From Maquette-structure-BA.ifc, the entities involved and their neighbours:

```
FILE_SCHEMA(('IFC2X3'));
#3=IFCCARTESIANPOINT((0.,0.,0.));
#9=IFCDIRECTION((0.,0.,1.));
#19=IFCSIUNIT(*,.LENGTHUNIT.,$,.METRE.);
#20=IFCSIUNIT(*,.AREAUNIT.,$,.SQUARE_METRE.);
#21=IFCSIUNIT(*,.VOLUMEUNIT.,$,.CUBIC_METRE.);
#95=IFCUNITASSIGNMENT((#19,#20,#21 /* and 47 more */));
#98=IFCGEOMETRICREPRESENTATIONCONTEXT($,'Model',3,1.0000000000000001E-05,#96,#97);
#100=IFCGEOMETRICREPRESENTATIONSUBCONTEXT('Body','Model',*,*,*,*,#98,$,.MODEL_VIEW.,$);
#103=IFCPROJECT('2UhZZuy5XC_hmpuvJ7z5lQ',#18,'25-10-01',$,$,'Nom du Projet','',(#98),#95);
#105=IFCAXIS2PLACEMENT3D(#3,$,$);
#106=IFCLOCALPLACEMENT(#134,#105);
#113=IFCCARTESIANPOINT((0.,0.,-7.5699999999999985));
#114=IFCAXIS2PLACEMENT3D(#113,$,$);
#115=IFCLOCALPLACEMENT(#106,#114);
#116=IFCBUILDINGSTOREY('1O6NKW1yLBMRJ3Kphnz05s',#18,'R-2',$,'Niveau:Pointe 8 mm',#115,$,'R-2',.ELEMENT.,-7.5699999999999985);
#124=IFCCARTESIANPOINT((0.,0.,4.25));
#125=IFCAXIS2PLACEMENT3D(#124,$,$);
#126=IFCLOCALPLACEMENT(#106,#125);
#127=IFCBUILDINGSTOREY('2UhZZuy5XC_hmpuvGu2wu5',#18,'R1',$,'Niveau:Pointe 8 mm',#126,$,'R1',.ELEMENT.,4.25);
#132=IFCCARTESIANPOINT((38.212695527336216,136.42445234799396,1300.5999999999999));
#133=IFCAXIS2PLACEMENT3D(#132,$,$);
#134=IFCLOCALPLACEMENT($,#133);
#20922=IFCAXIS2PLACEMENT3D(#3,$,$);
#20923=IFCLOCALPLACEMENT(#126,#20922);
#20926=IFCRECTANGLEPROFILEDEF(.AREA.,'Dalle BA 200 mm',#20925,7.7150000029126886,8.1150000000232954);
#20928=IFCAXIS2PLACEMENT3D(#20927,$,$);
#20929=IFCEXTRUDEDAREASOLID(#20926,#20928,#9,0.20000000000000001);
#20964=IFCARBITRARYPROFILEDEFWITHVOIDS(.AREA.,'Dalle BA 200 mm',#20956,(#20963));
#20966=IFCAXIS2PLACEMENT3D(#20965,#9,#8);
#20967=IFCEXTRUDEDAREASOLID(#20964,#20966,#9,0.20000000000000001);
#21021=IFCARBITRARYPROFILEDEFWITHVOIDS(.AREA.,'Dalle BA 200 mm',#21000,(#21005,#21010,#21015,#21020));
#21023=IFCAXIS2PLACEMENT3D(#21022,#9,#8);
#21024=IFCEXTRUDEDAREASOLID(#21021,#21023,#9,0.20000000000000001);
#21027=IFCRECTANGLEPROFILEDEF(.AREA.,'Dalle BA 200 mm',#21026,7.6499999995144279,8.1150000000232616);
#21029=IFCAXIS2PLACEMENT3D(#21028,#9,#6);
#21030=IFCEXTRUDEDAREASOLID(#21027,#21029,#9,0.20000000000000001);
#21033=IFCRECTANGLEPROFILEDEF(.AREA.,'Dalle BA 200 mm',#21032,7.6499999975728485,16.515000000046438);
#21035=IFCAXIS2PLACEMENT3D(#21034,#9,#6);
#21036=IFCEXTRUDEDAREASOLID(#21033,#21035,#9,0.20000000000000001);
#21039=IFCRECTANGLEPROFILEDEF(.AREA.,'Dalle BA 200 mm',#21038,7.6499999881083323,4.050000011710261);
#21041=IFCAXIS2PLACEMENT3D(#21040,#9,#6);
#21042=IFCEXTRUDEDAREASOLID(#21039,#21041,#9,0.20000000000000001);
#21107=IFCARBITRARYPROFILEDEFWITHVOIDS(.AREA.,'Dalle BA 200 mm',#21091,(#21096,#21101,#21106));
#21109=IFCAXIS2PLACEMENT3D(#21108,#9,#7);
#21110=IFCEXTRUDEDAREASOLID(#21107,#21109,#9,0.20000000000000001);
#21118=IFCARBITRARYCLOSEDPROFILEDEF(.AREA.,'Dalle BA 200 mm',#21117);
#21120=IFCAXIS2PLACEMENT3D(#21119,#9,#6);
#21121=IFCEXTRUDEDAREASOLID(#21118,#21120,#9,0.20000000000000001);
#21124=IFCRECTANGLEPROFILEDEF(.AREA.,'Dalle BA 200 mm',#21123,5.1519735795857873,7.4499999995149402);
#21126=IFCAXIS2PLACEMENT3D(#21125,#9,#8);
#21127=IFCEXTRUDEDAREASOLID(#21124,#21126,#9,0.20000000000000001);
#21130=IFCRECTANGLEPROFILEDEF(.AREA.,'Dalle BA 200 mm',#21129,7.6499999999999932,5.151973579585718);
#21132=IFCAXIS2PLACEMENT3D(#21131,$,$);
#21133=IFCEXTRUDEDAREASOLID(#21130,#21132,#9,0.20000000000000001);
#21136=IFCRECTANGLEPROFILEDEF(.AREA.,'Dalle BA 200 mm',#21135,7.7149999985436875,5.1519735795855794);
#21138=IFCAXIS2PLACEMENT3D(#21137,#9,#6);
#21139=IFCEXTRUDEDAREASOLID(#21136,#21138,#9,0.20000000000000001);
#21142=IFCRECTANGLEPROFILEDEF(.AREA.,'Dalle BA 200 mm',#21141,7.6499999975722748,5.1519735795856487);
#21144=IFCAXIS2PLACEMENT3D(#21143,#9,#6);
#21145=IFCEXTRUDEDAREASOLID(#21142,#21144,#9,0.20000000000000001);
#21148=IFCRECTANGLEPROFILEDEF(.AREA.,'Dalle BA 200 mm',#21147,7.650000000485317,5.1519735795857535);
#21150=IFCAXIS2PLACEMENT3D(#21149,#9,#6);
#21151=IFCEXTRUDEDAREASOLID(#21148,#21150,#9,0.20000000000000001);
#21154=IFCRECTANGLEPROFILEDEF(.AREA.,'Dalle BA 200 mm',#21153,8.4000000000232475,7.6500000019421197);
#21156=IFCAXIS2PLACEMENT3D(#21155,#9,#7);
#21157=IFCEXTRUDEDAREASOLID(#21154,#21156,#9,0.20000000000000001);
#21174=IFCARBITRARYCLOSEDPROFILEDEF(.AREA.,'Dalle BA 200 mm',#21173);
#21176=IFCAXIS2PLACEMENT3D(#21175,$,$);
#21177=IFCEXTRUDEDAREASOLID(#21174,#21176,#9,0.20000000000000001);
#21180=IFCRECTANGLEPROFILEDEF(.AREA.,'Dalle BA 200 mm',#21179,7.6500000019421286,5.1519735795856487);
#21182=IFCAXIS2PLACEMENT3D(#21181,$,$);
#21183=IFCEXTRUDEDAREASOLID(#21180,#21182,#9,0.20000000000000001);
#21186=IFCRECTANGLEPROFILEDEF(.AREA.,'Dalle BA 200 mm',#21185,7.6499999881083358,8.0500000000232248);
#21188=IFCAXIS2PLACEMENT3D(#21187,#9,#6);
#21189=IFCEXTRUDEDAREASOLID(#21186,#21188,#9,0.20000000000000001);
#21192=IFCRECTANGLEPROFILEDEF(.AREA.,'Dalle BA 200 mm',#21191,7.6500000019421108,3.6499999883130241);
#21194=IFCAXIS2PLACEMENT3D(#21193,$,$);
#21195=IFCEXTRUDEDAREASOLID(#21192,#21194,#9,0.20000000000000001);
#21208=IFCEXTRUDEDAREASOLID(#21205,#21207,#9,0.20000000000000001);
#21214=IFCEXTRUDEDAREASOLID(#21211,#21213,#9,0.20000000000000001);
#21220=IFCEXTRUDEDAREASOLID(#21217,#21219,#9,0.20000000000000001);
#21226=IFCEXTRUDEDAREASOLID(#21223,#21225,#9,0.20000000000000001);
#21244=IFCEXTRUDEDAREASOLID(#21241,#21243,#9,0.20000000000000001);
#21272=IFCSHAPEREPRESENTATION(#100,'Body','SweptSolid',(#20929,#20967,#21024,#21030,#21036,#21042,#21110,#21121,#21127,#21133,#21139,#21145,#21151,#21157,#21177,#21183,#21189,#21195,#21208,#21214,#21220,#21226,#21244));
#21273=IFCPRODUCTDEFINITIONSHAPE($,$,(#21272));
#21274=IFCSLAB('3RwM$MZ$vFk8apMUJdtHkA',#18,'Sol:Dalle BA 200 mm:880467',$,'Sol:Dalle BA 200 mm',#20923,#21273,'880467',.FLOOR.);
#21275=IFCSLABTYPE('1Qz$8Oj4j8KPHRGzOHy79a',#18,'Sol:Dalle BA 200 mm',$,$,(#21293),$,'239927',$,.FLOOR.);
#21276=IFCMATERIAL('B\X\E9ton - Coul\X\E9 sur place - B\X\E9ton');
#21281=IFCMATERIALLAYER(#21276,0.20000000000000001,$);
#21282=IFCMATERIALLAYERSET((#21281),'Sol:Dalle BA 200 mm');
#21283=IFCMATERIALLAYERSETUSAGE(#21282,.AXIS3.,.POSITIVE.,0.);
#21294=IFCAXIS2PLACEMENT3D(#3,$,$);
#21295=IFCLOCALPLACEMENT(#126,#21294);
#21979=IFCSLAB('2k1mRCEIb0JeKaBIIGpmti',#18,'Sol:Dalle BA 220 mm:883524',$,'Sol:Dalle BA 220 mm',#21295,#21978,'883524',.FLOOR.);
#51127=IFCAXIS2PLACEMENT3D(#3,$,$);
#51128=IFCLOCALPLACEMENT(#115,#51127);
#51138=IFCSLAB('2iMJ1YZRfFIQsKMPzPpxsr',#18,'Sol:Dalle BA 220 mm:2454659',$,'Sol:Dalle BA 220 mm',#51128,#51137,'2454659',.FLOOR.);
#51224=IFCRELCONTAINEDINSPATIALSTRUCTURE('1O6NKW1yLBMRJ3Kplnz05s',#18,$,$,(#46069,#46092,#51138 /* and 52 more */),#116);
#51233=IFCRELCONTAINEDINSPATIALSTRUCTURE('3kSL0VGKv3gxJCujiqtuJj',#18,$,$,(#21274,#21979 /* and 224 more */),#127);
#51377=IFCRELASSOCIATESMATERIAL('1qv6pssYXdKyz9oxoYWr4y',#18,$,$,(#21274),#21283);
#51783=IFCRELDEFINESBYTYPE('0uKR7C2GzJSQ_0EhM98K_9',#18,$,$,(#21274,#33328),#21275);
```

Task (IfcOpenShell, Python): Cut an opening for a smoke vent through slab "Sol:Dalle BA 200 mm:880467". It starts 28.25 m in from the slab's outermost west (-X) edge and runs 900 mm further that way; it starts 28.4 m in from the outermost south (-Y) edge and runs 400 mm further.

```python
import numpy as np
import ifcopenshell
import ifcopenshell.api.feature
import ifcopenshell.api.geometry
import ifcopenshell.api.root
import ifcopenshell.geom
import ifcopenshell.util.placement
import ifcopenshell.util.representation
import ifcopenshell.util.shape
import ifcopenshell.util.unit

model = ifcopenshell.open("Maquette-structure-BA.ifc")
unit_scale = ifcopenshell.util.unit.calculate_unit_scale(model)
settings = ifcopenshell.geom.settings()


def volume(element):
    """Net volume in cubic metres, openings subtracted."""
    shape = ifcopenshell.geom.create_shape(settings, element)
    return ifcopenshell.util.shape.get_volume(shape.geometry)


slab = model.by_id(21274)
before = volume(slab)

# Extent in the slab's own axes, in metres. The edges named are its -X and -Y sides.
slab_shape = ifcopenshell.geom.create_shape(settings, slab)
vertices = ifcopenshell.util.shape.get_vertices(slab_shape.geometry)
x_min, y_min, bottom = vertices.min(axis=0)
top = vertices[:, 2].max()

opening = ifcopenshell.api.root.create_entity(model, ifc_class="IfcOpeningElement", name="Smoke vent opening")
context = ifcopenshell.util.representation.get_context(model, "Model", "Body", "MODEL_VIEW")
width, depth = 0.9, 0.4
outline = [(0.0, 0.0), (width, 0.0), (width, depth), (0.0, depth), (0.0, 0.0)]
# Overshoot both faces by 50 mm so the cut is clean.
shape = ifcopenshell.api.geometry.add_slab_representation(
    model, context=context, depth=top - bottom + 0.1, polyline=outline
)
ifcopenshell.api.geometry.assign_representation(model, product=opening, representation=shape)

matrix = ifcopenshell.util.placement.get_local_placement(slab.ObjectPlacement)
matrix[:, 3] = matrix @ np.append(np.array([x_min + 28.25, y_min + 28.4, bottom - 0.05]) / unit_scale, 1.0)
ifcopenshell.api.geometry.edit_object_placement(model, product=opening, matrix=matrix, is_si=False)
ifcopenshell.api.feature.add_feature(model, feature=opening, element=slab)

after = volume(slab)

print(f"slab volume {before:.3f} -> {after:.3f} m3")

model.write("Maquette-structure-BA_edited.ifc")
```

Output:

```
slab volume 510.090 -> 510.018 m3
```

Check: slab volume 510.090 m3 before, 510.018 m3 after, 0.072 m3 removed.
